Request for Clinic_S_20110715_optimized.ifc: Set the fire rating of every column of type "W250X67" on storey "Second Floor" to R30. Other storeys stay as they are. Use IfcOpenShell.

First a look at what the model holds.

```python
import ifcopenshell
import ifcopenshell.util.element

model = ifcopenshell.open("Clinic_S_20110715_optimized.ifc")
print(model.schema)
storey = next(s for s in model.by_type("IfcBuildingStorey") if s.Name == "Second Floor")
columns = [e for e in ifcopenshell.util.element.get_decomposition(storey) if e.is_a("IfcColumn")]
seen = {}
for e in columns:
    element_type = ifcopenshell.util.element.get_type(e)
    key = (element_type.Name if element_type != e and element_type else None, ifcopenshell.util.element.get_pset(e, "Pset_ColumnCommon", "FireRating"))
    seen[key] = seen.get(key, 0) + 1
for (name, value), count in sorted(seen.items(), key=str):
    print(count, "x", name, "|", value)
```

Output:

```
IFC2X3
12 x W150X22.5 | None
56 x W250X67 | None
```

```python
import ifcopenshell
import ifcopenshell.api.pset
import ifcopenshell.util.element

model = ifcopenshell.open("Clinic_S_20110715_optimized.ifc")

storey = next(s for s in model.by_type("IfcBuildingStorey") if s.Name == "Second Floor")
columns = [e for e in ifcopenshell.util.element.get_decomposition(storey) if e.is_a("IfcColumn")]

count = 0
for e in columns:
    element_type = ifcopenshell.util.element.get_type(e)
    if element_type in (None, e) or element_type.Name != "W250X67":
        continue
    # add_pset returns the element's existing set when there is one.
    pset = ifcopenshell.api.pset.add_pset(model, product=e, name="Pset_ColumnCommon")
    ifcopenshell.api.pset.edit_pset(model, pset=pset, properties={"FireRating": "R30"})
    count += 1

print(count, "columns updated")

model.write("Clinic_S_20110715_optimized_rev.ifc")
```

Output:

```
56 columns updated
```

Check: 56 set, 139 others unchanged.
